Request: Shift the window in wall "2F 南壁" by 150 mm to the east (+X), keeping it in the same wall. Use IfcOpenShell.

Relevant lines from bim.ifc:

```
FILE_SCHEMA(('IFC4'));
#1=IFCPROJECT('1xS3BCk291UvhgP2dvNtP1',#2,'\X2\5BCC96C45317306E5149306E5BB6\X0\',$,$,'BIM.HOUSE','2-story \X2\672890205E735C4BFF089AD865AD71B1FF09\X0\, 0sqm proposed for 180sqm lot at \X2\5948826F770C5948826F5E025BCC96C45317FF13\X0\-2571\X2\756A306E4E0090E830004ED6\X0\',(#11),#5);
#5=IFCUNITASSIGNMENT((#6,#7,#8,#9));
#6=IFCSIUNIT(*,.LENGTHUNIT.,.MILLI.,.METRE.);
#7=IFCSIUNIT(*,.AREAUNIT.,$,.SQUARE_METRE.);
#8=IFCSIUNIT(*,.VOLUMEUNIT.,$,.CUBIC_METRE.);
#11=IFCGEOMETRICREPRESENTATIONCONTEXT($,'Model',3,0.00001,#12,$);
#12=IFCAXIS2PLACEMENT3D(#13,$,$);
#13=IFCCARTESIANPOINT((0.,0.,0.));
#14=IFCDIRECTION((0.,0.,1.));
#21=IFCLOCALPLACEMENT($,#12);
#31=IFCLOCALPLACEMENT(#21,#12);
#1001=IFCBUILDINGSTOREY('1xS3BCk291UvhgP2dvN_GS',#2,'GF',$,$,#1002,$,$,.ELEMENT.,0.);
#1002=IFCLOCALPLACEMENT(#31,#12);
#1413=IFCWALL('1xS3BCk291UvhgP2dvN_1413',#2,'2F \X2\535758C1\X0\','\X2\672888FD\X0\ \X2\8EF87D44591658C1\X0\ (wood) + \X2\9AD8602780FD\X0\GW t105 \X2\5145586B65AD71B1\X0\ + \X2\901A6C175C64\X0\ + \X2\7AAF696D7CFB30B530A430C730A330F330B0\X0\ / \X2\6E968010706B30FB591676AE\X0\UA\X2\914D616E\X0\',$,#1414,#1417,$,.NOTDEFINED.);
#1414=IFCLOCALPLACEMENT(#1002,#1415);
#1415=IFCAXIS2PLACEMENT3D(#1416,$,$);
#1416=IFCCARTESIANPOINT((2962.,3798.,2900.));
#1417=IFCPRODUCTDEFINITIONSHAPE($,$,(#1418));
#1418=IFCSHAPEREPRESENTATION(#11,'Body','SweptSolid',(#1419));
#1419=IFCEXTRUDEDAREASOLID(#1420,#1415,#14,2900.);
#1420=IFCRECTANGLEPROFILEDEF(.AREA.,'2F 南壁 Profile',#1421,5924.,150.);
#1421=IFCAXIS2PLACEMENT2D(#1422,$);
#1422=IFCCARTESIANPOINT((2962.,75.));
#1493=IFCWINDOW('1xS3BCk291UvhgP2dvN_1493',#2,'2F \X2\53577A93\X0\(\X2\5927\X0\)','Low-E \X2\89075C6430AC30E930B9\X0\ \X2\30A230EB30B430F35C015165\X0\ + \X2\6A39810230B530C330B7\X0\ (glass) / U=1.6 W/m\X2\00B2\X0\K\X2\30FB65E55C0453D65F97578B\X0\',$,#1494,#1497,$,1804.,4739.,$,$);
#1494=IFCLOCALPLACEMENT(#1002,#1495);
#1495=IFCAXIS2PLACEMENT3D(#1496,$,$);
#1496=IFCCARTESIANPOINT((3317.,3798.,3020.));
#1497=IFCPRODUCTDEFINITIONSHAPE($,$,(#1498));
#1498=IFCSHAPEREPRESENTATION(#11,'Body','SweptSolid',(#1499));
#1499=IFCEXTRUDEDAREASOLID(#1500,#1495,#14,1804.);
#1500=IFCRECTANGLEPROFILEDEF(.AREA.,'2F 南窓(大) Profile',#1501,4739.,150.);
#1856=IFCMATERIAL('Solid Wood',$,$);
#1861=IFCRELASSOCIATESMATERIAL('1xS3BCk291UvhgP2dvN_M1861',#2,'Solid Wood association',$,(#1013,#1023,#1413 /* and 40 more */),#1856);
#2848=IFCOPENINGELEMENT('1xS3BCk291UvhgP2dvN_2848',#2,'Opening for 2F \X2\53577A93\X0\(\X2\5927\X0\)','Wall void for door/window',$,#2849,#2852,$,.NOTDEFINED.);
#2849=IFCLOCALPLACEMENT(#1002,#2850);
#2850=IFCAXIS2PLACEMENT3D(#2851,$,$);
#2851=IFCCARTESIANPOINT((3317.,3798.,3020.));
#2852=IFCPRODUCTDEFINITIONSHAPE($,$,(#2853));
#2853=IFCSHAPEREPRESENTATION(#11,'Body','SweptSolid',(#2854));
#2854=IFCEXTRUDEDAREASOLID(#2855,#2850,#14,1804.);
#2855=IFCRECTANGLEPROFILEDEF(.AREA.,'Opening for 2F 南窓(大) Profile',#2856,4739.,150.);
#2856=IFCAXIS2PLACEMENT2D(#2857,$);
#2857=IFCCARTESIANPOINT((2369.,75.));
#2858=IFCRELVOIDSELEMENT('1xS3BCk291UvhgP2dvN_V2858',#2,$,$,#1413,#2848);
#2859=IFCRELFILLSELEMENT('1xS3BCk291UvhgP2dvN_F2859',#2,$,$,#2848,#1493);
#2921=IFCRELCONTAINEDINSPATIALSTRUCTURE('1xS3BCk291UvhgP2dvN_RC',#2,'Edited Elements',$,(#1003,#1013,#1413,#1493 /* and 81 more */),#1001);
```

```python
import ifcopenshell
import ifcopenshell.api.geometry
import ifcopenshell.util.placement

model = ifcopenshell.open("bim.ifc")

window = model.by_guid("1xS3BCk291UvhgP2dvN_1493")
opening = window.FillsVoids[0].RelatingOpeningElement
wall = opening.VoidsElements[0].RelatingBuildingElement

wall_matrix = ifcopenshell.util.placement.get_local_placement(wall.ObjectPlacement)
shift = wall_matrix[:3, 0] * 150.0
before = ifcopenshell.util.placement.get_local_placement(window.ObjectPlacement)[:3, 3].copy()

# The window is not placed relative to its opening, so move both.
for product in (opening, window):
    matrix = ifcopenshell.util.placement.get_local_placement(product.ObjectPlacement)
    matrix[:3, 3] += shift
    ifcopenshell.api.geometry.edit_object_placement(model, product=product, matrix=matrix, is_si=False)

after = ifcopenshell.util.placement.get_local_placement(window.ObjectPlacement)[:3, 3]
print("window moved by", (after - before).round(3) + 0.0)

model.write("bim_v2.ifc")
```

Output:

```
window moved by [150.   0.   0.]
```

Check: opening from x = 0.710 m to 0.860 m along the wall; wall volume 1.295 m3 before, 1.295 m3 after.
